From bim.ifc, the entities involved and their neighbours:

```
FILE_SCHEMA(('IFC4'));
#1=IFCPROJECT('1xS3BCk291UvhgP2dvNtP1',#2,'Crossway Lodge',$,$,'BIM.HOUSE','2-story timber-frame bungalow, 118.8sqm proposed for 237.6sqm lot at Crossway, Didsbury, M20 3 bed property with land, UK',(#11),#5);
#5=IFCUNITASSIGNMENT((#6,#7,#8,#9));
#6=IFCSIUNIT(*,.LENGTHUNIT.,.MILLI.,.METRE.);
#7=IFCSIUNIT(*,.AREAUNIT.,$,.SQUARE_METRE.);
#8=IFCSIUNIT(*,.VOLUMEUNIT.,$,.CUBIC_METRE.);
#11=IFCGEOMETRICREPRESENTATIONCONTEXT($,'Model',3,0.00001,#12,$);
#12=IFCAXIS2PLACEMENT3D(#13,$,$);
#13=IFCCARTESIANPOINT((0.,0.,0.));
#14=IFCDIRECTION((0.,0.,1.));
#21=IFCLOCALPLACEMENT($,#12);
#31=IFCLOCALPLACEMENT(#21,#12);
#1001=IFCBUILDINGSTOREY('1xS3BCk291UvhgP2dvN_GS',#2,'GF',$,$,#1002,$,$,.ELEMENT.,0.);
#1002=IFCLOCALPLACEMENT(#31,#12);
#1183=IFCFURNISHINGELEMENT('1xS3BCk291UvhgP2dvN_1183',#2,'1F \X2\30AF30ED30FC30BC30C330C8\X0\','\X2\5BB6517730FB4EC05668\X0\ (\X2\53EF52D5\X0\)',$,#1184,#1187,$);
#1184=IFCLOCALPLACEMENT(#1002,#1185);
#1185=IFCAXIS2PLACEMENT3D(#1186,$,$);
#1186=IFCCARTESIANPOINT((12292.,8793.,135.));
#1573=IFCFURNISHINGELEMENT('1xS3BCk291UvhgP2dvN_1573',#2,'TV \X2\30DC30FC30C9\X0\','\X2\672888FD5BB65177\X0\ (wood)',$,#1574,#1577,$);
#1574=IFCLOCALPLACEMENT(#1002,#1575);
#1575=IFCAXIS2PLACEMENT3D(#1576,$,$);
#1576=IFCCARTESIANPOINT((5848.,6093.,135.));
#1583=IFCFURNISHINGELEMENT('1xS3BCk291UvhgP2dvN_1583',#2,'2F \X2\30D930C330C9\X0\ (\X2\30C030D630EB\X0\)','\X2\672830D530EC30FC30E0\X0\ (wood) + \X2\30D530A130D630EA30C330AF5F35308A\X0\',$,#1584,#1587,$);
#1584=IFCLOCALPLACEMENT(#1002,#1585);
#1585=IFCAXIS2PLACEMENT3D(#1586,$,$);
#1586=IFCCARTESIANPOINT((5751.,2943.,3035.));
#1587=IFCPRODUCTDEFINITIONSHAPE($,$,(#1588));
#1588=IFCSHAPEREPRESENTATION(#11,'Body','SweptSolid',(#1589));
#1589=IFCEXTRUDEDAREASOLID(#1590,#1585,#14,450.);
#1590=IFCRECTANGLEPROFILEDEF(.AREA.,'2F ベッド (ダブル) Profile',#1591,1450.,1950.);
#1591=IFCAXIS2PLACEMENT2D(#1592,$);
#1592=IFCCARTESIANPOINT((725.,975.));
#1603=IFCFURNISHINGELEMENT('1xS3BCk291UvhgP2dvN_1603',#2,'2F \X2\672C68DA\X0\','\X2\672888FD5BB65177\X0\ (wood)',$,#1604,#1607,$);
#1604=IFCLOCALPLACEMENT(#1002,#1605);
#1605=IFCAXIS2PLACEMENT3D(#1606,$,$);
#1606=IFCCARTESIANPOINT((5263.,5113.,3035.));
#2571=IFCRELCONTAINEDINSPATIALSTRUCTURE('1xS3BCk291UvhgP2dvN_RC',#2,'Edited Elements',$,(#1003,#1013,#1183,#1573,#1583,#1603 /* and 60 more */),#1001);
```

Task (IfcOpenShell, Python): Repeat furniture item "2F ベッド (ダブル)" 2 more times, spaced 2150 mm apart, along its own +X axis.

```python
import ifcopenshell
import ifcopenshell.api.geometry
import ifcopenshell.api.root
import ifcopenshell.util.element
import ifcopenshell.util.placement
import ifcopenshell.util.unit

model = ifcopenshell.open("bim.ifc")
unit_scale = ifcopenshell.util.unit.calculate_unit_scale(model)


def reuse_history(source, copy):
    """copy_class also copies each property set's owner history, people and application; keep the originals."""
    for rel in copy.IsDefinedBy:
        if rel.is_a("IfcRelDefinesByProperties") and (history := rel.RelatingPropertyDefinition.OwnerHistory):
            rel.RelatingPropertyDefinition.OwnerHistory = source.OwnerHistory
            ifcopenshell.util.element.remove_deep2(model, history)


source = model.by_id(1583)
base = ifcopenshell.util.placement.get_local_placement(source.ObjectPlacement)
step = base[:3, 0] * 2.15 / unit_scale

for i in range(1, 3):
    copy = ifcopenshell.api.root.copy_class(model, product=source)
    copy.Representation = ifcopenshell.util.element.copy_deep(
        model, source.Representation, exclude=["IfcGeometricRepresentationContext", "IfcRepresentationMap"]
    )
    reuse_history(source, copy)
    matrix = base.copy()
    matrix[:3, 3] += i * step
    print("added at", matrix[:3, 3].round(3) + 0.0)
    ifcopenshell.api.geometry.edit_object_placement(model, product=copy, matrix=matrix, is_si=False)

model.write("bim_rev.ifc")
```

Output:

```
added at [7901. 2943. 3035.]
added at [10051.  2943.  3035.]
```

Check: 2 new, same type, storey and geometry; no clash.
